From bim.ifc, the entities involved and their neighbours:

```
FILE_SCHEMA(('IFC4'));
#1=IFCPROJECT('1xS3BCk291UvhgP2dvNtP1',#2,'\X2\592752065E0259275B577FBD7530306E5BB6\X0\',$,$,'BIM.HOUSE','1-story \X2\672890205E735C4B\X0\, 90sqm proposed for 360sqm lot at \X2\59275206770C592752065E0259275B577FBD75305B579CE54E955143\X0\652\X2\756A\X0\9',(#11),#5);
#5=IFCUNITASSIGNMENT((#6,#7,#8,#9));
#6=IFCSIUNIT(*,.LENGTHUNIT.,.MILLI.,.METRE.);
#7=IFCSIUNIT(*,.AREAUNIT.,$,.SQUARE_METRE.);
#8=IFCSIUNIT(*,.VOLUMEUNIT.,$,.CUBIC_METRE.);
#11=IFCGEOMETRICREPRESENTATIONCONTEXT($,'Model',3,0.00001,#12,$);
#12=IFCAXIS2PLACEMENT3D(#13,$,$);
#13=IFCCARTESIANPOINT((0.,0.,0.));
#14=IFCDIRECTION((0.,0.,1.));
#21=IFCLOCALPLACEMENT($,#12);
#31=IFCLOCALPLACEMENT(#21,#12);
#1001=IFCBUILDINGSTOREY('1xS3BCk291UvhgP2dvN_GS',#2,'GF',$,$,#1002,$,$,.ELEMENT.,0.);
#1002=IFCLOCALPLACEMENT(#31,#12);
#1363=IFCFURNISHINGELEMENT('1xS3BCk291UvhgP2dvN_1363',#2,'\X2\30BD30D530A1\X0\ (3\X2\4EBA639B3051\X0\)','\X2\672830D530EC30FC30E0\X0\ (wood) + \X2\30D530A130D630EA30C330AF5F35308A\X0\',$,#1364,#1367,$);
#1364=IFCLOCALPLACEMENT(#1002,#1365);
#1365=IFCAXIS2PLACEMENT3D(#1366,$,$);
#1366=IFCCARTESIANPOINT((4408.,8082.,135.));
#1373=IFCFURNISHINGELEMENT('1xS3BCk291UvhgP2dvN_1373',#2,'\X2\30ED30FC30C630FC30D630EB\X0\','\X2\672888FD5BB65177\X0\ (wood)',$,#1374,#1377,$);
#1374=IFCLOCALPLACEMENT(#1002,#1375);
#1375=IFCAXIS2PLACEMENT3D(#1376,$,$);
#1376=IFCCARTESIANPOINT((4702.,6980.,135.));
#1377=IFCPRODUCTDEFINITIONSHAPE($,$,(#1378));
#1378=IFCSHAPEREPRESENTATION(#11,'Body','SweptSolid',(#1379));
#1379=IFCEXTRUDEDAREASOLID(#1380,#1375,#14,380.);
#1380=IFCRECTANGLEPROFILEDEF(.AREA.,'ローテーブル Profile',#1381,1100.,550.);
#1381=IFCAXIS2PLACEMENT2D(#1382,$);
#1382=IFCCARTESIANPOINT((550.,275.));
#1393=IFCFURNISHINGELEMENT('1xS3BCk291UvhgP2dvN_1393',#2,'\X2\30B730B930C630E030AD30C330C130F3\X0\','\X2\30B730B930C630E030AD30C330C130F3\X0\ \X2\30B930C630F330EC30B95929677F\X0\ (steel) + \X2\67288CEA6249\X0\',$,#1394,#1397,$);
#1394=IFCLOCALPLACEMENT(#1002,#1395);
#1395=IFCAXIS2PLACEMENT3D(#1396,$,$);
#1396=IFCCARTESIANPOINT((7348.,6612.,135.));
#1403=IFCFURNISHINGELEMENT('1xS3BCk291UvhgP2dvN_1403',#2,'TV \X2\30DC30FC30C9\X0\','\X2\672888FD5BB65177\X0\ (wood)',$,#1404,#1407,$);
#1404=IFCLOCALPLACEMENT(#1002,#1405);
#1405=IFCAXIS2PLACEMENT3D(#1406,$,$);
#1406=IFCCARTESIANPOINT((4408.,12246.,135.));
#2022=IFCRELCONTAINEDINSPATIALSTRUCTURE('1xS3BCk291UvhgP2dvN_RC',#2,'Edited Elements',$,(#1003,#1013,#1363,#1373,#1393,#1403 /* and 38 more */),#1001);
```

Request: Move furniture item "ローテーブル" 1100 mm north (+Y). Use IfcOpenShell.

```python
import ifcopenshell
import ifcopenshell.api.geometry
import ifcopenshell.util.placement
import ifcopenshell.util.unit

model = ifcopenshell.open("bim.ifc")
unit_scale = ifcopenshell.util.unit.calculate_unit_scale(model)

item = model.by_guid("1xS3BCk291UvhgP2dvN_1373")
matrix = ifcopenshell.util.placement.get_local_placement(item.ObjectPlacement)
matrix[1, 3] += 1.1 / unit_scale
ifcopenshell.api.geometry.edit_object_placement(model, product=item, matrix=matrix, is_si=False)

print(ifcopenshell.util.placement.get_local_placement(item.ObjectPlacement).round(3) + 0.0)

model.write("bim_v2.ifc")
```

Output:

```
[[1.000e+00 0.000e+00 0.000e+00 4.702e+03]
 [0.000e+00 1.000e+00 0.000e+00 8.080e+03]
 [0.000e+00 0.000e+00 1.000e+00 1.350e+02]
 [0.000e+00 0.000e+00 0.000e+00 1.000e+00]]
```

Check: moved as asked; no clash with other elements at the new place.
